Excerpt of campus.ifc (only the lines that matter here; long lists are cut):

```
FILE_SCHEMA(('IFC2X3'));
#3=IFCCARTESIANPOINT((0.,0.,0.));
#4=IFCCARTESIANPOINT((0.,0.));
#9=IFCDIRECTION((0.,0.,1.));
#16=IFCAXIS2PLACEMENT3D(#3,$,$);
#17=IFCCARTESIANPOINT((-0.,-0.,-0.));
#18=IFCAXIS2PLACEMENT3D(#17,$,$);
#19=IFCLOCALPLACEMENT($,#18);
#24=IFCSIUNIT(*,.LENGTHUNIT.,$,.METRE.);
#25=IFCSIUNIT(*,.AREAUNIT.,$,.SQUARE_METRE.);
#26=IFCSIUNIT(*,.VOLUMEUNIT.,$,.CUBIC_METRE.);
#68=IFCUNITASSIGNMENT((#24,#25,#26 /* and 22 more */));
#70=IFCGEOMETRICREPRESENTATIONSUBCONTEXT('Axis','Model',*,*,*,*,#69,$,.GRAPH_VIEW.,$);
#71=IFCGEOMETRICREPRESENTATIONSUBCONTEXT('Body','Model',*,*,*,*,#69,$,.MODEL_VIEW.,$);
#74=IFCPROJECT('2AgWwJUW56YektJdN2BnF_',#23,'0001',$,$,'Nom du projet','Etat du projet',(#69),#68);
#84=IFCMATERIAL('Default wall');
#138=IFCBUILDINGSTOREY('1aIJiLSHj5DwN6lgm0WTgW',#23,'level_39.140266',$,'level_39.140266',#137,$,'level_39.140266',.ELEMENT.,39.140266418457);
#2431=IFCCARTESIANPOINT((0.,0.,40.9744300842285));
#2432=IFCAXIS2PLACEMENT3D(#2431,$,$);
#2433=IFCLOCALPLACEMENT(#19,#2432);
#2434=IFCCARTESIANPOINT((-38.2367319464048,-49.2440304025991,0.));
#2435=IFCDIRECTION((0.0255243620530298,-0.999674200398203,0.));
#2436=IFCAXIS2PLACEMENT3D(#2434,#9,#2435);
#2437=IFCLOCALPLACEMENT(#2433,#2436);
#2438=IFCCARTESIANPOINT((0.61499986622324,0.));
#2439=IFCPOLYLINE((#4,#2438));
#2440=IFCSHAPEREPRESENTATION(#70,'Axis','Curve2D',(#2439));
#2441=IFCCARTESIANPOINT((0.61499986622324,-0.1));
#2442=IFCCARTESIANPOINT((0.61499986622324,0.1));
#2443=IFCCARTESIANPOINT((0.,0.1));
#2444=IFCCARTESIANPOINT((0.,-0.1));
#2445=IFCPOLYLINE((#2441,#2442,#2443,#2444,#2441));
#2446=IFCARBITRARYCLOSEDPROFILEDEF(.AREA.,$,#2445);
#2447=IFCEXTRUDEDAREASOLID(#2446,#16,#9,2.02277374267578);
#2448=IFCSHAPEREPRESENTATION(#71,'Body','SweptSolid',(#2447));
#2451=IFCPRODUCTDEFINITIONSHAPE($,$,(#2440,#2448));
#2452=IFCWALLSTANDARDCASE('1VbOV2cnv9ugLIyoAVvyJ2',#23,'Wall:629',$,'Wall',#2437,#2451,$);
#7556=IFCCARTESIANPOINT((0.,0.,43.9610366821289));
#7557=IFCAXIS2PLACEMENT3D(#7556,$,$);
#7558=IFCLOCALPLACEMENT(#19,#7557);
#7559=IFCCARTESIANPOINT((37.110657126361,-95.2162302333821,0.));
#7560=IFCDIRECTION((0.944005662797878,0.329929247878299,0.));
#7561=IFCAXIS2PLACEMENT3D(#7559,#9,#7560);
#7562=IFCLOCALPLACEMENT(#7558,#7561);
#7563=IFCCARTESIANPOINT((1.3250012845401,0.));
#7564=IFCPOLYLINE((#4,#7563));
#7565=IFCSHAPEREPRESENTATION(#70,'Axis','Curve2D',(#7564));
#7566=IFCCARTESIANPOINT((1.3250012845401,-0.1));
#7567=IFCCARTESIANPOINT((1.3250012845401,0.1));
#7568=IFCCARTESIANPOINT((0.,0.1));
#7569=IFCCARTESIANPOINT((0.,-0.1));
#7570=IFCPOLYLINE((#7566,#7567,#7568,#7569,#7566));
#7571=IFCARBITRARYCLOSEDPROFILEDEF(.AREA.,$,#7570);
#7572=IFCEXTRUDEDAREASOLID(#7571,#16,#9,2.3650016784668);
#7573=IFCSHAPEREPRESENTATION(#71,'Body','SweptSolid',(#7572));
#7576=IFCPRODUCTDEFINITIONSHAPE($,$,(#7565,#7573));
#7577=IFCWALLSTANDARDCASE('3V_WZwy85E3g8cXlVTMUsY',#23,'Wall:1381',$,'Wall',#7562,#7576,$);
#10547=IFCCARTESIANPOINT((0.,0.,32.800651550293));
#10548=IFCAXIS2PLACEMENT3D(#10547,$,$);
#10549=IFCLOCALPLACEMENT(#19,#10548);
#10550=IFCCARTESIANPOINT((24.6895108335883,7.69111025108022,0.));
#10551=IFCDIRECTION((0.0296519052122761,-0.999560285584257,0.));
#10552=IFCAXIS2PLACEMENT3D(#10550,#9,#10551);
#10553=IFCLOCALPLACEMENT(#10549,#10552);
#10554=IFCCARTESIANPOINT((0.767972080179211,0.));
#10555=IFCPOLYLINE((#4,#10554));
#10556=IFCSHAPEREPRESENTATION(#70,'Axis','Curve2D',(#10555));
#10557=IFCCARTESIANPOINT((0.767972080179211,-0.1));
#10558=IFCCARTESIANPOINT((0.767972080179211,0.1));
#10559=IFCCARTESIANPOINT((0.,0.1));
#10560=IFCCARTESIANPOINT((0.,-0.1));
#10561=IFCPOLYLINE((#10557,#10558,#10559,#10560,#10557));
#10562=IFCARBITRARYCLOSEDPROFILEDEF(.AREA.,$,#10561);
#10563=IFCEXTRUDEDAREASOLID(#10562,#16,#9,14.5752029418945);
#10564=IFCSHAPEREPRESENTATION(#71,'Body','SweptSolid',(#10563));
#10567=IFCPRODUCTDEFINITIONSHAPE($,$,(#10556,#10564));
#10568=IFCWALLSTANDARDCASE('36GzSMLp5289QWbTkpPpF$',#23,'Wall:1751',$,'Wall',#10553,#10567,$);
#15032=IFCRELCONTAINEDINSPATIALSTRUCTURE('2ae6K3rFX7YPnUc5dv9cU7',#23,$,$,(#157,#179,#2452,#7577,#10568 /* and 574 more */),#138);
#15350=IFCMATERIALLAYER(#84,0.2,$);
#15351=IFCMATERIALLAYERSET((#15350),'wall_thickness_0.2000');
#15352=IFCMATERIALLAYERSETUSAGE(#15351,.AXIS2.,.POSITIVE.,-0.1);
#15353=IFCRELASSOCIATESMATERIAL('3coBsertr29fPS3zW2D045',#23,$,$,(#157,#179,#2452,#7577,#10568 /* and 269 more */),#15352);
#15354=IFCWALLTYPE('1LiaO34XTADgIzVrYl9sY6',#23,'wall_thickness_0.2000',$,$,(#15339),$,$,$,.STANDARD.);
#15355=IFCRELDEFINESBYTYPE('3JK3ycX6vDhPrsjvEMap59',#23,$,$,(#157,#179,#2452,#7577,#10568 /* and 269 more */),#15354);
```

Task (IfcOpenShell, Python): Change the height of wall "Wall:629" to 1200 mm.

```python
import ifcopenshell
import ifcopenshell.geom
import ifcopenshell.util.representation
import ifcopenshell.util.shape

model = ifcopenshell.open("campus.ifc")
settings = ifcopenshell.geom.settings()


def volume(element):
    """Net volume in cubic metres, openings subtracted."""
    shape = ifcopenshell.geom.create_shape(settings, element)
    return ifcopenshell.util.shape.get_volume(shape.geometry)


wall = model.by_id(2452)
before = volume(wall)

body = ifcopenshell.util.representation.get_representation(wall, "Model", "Body")
solid = body.Items[0]
old_height = solid.Depth
solid.Depth = 1.2
after = volume(wall)

print(f"height {old_height:g} -> {solid.Depth:g}, volume {before:.3f} -> {after:.3f} m3")

model.write("campus_edited.ifc")
```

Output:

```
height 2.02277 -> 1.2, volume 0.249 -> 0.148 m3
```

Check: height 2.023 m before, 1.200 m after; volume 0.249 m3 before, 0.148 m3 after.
